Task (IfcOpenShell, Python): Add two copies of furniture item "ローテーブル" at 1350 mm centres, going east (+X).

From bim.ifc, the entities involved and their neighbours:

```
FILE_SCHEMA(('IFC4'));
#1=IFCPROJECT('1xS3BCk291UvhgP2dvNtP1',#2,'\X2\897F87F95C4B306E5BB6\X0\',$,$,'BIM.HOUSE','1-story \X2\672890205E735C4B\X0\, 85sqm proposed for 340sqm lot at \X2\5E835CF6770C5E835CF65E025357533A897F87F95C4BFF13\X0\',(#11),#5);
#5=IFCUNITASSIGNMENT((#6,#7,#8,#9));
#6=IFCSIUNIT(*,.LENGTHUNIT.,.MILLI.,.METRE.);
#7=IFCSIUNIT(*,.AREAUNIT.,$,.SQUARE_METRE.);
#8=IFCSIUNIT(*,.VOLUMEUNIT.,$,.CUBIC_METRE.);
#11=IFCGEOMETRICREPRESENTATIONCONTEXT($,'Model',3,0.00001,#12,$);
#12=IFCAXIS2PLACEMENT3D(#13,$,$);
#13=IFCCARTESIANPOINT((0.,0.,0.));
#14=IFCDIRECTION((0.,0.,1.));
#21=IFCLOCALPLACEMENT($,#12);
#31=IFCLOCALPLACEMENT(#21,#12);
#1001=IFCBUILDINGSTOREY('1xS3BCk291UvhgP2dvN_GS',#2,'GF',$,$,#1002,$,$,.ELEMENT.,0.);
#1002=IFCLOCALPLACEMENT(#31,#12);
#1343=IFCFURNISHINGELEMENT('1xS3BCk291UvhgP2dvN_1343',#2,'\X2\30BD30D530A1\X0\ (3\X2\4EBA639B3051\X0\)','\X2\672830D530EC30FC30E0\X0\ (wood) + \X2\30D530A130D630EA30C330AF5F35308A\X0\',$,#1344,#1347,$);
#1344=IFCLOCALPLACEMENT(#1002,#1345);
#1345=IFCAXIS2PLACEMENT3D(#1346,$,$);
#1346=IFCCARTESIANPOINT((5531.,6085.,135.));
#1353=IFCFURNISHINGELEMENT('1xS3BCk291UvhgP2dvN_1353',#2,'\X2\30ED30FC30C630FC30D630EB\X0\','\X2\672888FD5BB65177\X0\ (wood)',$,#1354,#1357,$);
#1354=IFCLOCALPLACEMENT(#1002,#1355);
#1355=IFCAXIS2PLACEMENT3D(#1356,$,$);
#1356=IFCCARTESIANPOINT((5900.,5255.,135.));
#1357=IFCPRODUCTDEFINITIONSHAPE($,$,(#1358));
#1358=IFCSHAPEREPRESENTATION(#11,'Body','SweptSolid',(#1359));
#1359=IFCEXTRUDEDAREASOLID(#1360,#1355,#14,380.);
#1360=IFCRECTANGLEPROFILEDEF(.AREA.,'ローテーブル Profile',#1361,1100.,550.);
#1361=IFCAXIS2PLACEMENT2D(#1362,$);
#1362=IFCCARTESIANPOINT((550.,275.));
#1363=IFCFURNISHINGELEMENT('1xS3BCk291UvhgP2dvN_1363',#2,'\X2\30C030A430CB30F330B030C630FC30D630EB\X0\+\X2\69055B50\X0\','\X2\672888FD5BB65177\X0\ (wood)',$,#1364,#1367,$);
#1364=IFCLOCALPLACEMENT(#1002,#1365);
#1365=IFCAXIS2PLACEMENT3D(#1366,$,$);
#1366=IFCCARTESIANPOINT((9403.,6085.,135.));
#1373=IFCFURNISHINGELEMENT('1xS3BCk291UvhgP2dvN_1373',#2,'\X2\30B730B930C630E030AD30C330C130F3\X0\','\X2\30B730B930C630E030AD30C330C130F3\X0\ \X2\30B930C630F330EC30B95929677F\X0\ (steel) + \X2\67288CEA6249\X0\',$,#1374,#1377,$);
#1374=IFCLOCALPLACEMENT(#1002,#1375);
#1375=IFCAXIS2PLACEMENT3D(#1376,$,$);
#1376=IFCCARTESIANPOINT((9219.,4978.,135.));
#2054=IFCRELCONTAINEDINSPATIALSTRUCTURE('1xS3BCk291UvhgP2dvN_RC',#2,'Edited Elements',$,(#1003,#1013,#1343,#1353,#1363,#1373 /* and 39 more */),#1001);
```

```python
import numpy as np
import ifcopenshell
import ifcopenshell.api.geometry
import ifcopenshell.api.root
import ifcopenshell.util.element
import ifcopenshell.util.placement

model = ifcopenshell.open("bim.ifc")


def reuse_history(source, copy):
    """copy_class also copies each property set's owner history, people and application; keep the originals."""
    for rel in copy.IsDefinedBy:
        if rel.is_a("IfcRelDefinesByProperties") and (history := rel.RelatingPropertyDefinition.OwnerHistory):
            rel.RelatingPropertyDefinition.OwnerHistory = source.OwnerHistory
            ifcopenshell.util.element.remove_deep2(model, history)


source = model.by_id(1353)
base = ifcopenshell.util.placement.get_local_placement(source.ObjectPlacement)
step = np.array([1.0, 0.0, 0.0]) * 1350.0

for i in range(1, 3):
    copy = ifcopenshell.api.root.copy_class(model, product=source)
    copy.Representation = ifcopenshell.util.element.copy_deep(
        model, source.Representation, exclude=["IfcGeometricRepresentationContext", "IfcRepresentationMap"]
    )
    reuse_history(source, copy)
    matrix = base.copy()
    matrix[:3, 3] += i * step
    print("added at", matrix[:3, 3].round(3) + 0.0)
    ifcopenshell.api.geometry.edit_object_placement(model, product=copy, matrix=matrix, is_si=False)

model.write("bim_updated.ifc")
```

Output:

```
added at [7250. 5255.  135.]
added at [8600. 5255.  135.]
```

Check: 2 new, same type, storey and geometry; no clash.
